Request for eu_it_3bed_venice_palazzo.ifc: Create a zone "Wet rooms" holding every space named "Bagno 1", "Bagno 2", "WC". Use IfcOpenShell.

First a look at what the model holds.

```python
import ifcopenshell

model = ifcopenshell.open("eu_it_3bed_venice_palazzo.ifc")
print(model.schema)
seen = {}
for space in model.by_type("IfcSpace"):
    seen[space.LongName] = seen.get(space.LongName, 0) + 1
for name, count in sorted(seen.items(), key=str):
    print(count, "x", name)
print("zones:", [z.Name for z in model.by_type("IfcZone")][:20])
```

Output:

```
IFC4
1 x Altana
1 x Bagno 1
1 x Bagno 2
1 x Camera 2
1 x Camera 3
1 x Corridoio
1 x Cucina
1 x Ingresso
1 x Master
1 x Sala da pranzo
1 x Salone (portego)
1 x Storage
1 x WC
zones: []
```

```python
import ifcopenshell
import ifcopenshell.api.group
import ifcopenshell.api.root

model = ifcopenshell.open("eu_it_3bed_venice_palazzo.ifc")

names = {"Bagno 1", "Bagno 2", "WC"}
spaces = [s for s in model.by_type("IfcSpace") if s.LongName in names]

zone = ifcopenshell.api.root.create_entity(model, ifc_class="IfcZone", name="Wet rooms")
ifcopenshell.api.group.assign_group(model, products=spaces, group=zone)
print(len(spaces), "spaces in", zone.Name)

model.write("eu_it_3bed_venice_palazzo-out.ifc")
```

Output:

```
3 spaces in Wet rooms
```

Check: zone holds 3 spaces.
